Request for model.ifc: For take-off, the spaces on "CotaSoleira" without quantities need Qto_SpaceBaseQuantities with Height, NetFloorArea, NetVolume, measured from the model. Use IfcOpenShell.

First a look at what the model holds.

```python
import ifcopenshell
import ifcopenshell.util.element
import ifcopenshell.util.unit

model = ifcopenshell.open("model.ifc")
print(model.schema)
for unit_type in ("LENGTHUNIT", "AREAUNIT", "VOLUMEUNIT"):
    print(unit_type, ifcopenshell.util.unit.calculate_unit_scale(model, unit_type))
storey = next(s for s in model.by_type("IfcBuildingStorey") if s.Name == "CotaSoleira")
spaces = [e for e in ifcopenshell.util.element.get_decomposition(storey) if e.is_a("IfcSpace")]
for e in sorted(spaces, key=lambda e: e.id()):
    print(e.id(), e.is_a(), e.Name, list(ifcopenshell.util.element.get_psets(e, qtos_only=True)), sep=" | ")
```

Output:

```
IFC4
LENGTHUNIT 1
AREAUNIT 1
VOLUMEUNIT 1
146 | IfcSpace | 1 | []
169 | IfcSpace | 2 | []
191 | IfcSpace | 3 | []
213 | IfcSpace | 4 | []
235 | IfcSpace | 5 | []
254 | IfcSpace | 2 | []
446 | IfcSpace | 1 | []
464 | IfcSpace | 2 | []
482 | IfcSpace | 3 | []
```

```python
import ifcopenshell
import ifcopenshell.api.pset
import ifcopenshell.geom
import ifcopenshell.util.element
import ifcopenshell.util.shape
import ifcopenshell.util.unit

model = ifcopenshell.open("model.ifc")
unit_scale = ifcopenshell.util.unit.calculate_unit_scale(model)
area_scale = ifcopenshell.util.unit.calculate_unit_scale(model, "AREAUNIT")
volume_scale = ifcopenshell.util.unit.calculate_unit_scale(model, "VOLUMEUNIT")
settings = ifcopenshell.geom.settings()

storey = next(s for s in model.by_type("IfcBuildingStorey") if s.Name == "CotaSoleira")
spaces = [e for e in ifcopenshell.util.element.get_decomposition(storey) if e.is_a("IfcSpace")]

for e in sorted(spaces, key=lambda e: e.id()):
    if ifcopenshell.util.element.get_psets(e, qtos_only=True, should_inherit=False):
        continue
    # Geometry comes back in metres, in the element's own axes.
    shape = ifcopenshell.geom.create_shape(settings, e)
    values = {
        "Height": ifcopenshell.util.shape.get_z(shape.geometry) / unit_scale,
        "NetFloorArea": ifcopenshell.util.shape.get_footprint_area(shape.geometry) / area_scale,
        "NetVolume": ifcopenshell.util.shape.get_volume(shape.geometry) / volume_scale,
    }
    qto = ifcopenshell.api.pset.add_qto(model, product=e, name="Qto_SpaceBaseQuantities")
    ifcopenshell.api.pset.edit_qto(model, qto=qto, properties=values)
    print(e.id(), {k: round(v, 3) for k, v in values.items()})

model.write("model_edited.ifc")
```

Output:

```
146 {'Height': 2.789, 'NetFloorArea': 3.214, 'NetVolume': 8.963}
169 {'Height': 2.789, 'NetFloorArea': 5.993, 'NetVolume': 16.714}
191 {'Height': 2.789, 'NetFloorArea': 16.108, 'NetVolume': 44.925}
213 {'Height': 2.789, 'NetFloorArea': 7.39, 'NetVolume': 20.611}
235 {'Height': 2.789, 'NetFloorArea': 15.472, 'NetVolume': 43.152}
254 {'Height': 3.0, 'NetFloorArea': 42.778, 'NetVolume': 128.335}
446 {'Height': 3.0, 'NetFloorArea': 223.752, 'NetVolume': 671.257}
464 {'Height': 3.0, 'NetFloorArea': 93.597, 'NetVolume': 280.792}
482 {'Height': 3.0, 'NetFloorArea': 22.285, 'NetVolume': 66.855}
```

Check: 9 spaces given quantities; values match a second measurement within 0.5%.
